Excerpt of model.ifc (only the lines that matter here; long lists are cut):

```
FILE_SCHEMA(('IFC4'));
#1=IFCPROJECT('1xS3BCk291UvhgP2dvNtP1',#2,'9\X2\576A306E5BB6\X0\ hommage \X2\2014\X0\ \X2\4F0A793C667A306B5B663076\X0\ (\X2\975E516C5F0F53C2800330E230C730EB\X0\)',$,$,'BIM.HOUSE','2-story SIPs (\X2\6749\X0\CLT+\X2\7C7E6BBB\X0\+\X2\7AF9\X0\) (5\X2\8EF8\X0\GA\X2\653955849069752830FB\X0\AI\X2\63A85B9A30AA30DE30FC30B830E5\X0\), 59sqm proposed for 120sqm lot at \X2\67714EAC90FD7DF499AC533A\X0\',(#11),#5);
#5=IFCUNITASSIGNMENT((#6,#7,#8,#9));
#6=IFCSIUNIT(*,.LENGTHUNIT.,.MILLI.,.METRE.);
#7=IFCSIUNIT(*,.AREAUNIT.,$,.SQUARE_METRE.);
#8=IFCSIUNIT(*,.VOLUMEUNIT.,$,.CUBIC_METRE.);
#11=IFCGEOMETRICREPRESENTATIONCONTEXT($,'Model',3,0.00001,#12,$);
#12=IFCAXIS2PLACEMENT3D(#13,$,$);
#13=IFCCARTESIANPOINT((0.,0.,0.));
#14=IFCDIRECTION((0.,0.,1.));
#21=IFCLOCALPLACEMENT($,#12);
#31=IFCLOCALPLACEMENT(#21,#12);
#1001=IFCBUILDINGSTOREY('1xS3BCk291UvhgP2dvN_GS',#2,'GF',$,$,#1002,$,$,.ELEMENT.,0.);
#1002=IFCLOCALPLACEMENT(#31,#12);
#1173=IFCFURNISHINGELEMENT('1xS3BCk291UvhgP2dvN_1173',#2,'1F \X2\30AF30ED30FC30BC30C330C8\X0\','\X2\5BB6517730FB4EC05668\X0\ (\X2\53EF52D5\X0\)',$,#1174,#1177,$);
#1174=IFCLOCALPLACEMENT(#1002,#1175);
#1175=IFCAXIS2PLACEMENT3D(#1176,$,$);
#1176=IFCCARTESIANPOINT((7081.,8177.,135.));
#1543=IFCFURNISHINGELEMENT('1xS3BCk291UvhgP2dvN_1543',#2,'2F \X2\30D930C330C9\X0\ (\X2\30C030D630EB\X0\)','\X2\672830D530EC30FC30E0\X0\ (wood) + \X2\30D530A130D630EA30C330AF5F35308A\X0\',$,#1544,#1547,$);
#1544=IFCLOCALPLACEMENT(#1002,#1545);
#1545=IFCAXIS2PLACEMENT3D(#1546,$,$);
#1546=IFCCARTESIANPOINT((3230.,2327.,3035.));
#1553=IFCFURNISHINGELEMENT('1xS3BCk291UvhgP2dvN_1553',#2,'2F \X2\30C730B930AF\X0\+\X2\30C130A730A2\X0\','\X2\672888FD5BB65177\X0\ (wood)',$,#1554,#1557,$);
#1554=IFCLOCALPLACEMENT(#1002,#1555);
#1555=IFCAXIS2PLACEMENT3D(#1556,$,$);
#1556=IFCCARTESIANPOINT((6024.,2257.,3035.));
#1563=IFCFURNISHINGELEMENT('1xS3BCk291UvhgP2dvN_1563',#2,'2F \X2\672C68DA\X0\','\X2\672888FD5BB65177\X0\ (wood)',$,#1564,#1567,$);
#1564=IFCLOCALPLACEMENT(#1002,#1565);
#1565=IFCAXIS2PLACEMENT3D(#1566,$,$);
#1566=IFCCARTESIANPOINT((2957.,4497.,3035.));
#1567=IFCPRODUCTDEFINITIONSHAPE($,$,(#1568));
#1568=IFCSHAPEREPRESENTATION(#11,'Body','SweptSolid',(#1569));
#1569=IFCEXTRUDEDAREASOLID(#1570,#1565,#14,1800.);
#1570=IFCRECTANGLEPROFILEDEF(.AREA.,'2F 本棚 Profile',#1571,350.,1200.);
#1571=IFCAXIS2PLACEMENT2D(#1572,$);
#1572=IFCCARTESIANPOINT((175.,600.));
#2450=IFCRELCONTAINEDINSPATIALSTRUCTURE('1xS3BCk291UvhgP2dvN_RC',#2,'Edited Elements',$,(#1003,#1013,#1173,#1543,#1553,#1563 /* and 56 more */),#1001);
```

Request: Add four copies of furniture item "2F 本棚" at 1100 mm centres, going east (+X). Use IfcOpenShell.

```python
import numpy as np
import ifcopenshell
import ifcopenshell.api.geometry
import ifcopenshell.api.root
import ifcopenshell.util.element
import ifcopenshell.util.placement

model = ifcopenshell.open("model.ifc")


def reuse_history(source, copy):
    """copy_class also copies each property set's owner history, people and application; keep the originals."""
    for rel in copy.IsDefinedBy:
        if rel.is_a("IfcRelDefinesByProperties") and (history := rel.RelatingPropertyDefinition.OwnerHistory):
            rel.RelatingPropertyDefinition.OwnerHistory = source.OwnerHistory
            ifcopenshell.util.element.remove_deep2(model, history)


source = model.by_id(1563)
base = ifcopenshell.util.placement.get_local_placement(source.ObjectPlacement)
step = np.array([1.0, 0.0, 0.0]) * 1100.0

for i in range(1, 5):
    copy = ifcopenshell.api.root.copy_class(model, product=source)
    copy.Representation = ifcopenshell.util.element.copy_deep(
        model, source.Representation, exclude=["IfcGeometricRepresentationContext", "IfcRepresentationMap"]
    )
    reuse_history(source, copy)
    matrix = base.copy()
    matrix[:3, 3] += i * step
    print("added at", matrix[:3, 3].round(3) + 0.0)
    ifcopenshell.api.geometry.edit_object_placement(model, product=copy, matrix=matrix, is_si=False)

model.write("model_edited.ifc")
```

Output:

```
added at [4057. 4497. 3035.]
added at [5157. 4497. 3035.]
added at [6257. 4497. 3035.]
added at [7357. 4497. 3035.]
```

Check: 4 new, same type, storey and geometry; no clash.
